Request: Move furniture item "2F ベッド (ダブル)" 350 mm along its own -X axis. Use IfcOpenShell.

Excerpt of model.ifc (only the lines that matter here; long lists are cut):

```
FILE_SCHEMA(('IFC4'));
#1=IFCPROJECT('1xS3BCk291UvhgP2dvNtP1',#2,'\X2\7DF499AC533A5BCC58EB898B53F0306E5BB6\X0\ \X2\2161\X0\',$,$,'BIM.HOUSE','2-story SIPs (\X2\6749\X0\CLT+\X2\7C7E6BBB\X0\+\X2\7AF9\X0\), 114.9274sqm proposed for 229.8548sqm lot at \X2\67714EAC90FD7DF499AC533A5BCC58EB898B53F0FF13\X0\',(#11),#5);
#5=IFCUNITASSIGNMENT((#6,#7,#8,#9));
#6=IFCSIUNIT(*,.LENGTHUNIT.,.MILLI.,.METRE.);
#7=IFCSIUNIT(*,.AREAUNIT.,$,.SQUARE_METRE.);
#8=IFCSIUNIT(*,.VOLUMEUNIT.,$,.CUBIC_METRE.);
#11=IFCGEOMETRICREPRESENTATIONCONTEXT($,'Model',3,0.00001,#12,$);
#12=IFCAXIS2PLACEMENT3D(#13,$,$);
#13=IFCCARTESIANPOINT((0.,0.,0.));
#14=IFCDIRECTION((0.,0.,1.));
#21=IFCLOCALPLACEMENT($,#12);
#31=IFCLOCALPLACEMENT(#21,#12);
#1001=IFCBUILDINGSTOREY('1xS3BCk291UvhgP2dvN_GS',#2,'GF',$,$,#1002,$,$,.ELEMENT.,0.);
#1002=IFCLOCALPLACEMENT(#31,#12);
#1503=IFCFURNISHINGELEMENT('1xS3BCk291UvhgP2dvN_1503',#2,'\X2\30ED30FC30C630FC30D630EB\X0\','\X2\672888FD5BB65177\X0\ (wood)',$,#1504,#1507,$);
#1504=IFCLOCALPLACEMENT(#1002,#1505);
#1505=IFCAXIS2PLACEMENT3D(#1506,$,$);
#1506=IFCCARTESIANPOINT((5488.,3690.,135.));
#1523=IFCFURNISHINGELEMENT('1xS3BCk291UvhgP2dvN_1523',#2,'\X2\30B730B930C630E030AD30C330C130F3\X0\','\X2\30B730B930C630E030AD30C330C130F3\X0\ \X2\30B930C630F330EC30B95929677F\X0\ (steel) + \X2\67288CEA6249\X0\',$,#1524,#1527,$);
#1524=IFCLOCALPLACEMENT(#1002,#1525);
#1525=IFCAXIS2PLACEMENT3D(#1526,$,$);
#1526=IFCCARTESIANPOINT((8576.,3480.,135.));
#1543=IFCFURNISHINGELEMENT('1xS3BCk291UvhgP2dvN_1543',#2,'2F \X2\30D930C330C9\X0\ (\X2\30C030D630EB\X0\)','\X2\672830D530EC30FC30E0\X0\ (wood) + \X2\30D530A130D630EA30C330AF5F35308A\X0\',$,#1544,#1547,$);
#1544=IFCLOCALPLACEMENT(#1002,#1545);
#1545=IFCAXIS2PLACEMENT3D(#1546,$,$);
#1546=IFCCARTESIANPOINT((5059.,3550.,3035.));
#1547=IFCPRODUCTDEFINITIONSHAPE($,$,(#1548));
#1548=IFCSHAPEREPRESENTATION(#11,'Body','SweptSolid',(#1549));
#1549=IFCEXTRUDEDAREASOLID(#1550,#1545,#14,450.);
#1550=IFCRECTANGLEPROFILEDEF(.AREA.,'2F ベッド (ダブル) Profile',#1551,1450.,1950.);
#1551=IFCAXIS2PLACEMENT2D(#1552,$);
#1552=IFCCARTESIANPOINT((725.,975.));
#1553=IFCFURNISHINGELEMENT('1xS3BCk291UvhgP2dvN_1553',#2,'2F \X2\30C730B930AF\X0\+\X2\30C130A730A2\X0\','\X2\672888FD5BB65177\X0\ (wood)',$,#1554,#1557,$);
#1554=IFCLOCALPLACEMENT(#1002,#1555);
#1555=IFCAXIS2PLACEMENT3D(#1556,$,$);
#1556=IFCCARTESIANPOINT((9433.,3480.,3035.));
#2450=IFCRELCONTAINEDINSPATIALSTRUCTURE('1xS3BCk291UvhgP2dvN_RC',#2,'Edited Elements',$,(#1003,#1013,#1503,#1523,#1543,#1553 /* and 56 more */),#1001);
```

```python
import ifcopenshell
import ifcopenshell.api.geometry
import ifcopenshell.util.placement
import ifcopenshell.util.unit

model = ifcopenshell.open("model.ifc")
unit_scale = ifcopenshell.util.unit.calculate_unit_scale(model)

item = model.by_guid("1xS3BCk291UvhgP2dvN_1543")
matrix = ifcopenshell.util.placement.get_local_placement(item.ObjectPlacement)
matrix[:3, 3] -= matrix[:3, 0] * 0.35 / unit_scale
ifcopenshell.api.geometry.edit_object_placement(model, product=item, matrix=matrix, is_si=False)

print(ifcopenshell.util.placement.get_local_placement(item.ObjectPlacement).round(3) + 0.0)

model.write("model_edited.ifc")
```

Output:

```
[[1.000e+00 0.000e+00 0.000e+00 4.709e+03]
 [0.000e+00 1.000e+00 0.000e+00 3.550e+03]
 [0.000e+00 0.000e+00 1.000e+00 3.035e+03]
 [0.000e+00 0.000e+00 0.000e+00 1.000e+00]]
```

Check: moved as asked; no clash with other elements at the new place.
